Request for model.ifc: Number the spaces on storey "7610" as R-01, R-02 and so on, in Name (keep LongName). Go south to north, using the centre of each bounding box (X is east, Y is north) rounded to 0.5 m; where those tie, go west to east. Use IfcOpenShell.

First a look at what the model holds.

```python
import ifcopenshell
import ifcopenshell.util.element
import ifcopenshell.util.placement

model = ifcopenshell.open("model.ifc")
print(model.schema)
storey = next(s for s in model.by_type("IfcBuildingStorey") if s.Name == "7610")
spaces = [e for e in ifcopenshell.util.element.get_decomposition(storey) if e.is_a("IfcSpace")]
for e in sorted(spaces, key=lambda e: e.id()):
    origin = ifcopenshell.util.placement.get_local_placement(e.ObjectPlacement)[:3, 3]
    print(e.id(), e.Name, e.LongName, origin.round(2) + 0.0, sep=" | ")
```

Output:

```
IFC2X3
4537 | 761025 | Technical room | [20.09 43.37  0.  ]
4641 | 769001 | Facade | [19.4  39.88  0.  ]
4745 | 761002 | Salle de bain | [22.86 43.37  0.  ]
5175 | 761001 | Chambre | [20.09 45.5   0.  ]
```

```python
import ifcopenshell
import ifcopenshell.geom
import ifcopenshell.util.element
import ifcopenshell.util.shape

model = ifcopenshell.open("model.ifc")
settings = ifcopenshell.geom.settings()
settings.set("use-world-coords", True)


def centre(element):
    shape = ifcopenshell.geom.create_shape(settings, element)
    return ifcopenshell.util.shape.get_bbox_centroid(shape.geometry)


storey = next(s for s in model.by_type("IfcBuildingStorey") if s.Name == "7610")
spaces = [e for e in ifcopenshell.util.element.get_decomposition(storey) if e.is_a("IfcSpace")]

# Insertion points can sit at a corner or the storey origin, so sort by the geometry (in metres).
centres = {e: centre(e) for e in spaces}
spaces.sort(key=lambda e: (round(centres[e][1] / 0.5), centres[e][0]))

for i, e in enumerate(spaces, start=1):
    number = f"R-{i:02d}"
    e.Name = number
    print(e.id(), number)

model.write("model_updated.ifc")
```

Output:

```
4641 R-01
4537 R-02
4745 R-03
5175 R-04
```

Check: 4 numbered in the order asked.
